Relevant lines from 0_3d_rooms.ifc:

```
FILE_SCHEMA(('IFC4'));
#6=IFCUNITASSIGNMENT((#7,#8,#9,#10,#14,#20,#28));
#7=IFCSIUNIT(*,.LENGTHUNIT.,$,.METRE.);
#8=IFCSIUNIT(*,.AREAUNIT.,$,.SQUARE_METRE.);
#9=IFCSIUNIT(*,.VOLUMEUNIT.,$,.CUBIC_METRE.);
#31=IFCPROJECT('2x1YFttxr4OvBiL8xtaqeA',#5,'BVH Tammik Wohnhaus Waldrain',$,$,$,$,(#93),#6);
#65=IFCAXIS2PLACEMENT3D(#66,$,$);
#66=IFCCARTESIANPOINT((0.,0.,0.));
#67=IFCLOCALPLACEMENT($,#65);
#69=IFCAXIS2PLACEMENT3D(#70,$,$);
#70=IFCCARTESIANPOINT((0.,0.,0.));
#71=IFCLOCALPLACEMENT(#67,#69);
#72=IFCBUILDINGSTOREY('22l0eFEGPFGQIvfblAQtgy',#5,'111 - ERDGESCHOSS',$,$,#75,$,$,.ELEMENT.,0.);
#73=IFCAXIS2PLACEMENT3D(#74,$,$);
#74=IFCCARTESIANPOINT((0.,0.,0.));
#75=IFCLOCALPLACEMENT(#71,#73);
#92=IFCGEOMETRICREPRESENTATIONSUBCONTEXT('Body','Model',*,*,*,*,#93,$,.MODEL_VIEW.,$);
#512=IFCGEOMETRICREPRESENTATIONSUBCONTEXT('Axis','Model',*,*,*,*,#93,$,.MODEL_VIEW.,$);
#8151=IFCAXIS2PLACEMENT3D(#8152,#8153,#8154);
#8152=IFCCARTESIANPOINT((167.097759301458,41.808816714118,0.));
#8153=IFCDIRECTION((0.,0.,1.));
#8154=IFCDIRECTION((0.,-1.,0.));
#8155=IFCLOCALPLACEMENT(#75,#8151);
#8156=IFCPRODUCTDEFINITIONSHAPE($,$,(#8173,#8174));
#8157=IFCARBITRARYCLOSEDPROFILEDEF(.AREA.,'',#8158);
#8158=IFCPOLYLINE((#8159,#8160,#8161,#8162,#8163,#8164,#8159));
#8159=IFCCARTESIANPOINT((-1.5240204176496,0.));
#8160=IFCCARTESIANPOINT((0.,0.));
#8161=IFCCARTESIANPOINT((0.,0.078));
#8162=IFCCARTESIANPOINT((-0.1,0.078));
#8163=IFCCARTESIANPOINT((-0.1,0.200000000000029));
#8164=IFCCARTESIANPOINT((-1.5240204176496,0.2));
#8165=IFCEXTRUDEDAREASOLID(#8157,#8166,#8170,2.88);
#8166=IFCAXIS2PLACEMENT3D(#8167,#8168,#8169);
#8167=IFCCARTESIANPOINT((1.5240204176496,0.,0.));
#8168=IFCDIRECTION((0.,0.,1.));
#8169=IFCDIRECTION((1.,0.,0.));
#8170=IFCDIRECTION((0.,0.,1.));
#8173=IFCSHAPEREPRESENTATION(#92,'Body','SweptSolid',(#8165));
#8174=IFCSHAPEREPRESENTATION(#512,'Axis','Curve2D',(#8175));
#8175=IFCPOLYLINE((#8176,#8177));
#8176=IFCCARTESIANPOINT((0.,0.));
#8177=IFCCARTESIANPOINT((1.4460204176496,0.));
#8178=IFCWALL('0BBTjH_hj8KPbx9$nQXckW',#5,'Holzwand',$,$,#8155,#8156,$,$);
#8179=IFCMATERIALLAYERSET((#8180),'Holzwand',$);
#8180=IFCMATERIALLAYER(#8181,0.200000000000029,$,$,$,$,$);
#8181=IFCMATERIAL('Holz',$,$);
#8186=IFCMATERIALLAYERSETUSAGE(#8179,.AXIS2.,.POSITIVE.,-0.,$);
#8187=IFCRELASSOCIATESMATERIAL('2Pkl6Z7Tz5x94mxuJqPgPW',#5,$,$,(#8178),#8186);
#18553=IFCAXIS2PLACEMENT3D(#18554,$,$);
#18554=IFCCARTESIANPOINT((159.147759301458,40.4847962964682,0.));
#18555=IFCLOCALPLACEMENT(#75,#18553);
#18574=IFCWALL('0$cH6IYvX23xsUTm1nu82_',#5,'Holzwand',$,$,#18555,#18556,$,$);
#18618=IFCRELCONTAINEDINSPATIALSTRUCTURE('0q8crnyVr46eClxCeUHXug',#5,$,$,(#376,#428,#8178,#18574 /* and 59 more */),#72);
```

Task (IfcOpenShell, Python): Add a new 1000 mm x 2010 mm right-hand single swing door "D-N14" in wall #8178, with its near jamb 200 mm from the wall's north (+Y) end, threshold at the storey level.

```python
import numpy as np
import ifcopenshell
import ifcopenshell.api.feature
import ifcopenshell.api.geometry
import ifcopenshell.api.root
import ifcopenshell.api.spatial
import ifcopenshell.geom
import ifcopenshell.util.element
import ifcopenshell.util.placement
import ifcopenshell.util.representation
import ifcopenshell.util.shape
import ifcopenshell.util.unit

model = ifcopenshell.open("0_3d_rooms.ifc")
unit_scale = ifcopenshell.util.unit.calculate_unit_scale(model)
settings = ifcopenshell.geom.settings()


def volume(element):
    """Net volume in cubic metres, openings subtracted."""
    shape = ifcopenshell.geom.create_shape(settings, element)
    return ifcopenshell.util.shape.get_volume(shape.geometry)


wall = model.by_guid("0BBTjH_hj8KPbx9$nQXckW")
storey = ifcopenshell.util.element.get_container(wall, ifc_class="IfcBuildingStorey")
context = ifcopenshell.util.representation.get_context(model, "Model", "Body", "MODEL_VIEW")
before = volume(wall)

width, height, from_end, sill = 1, 2.01, 0.2, 0.0  # metres

# The wall runs along its own X axis, and the end named is its -X end.
wall_shape = ifcopenshell.geom.create_shape(settings, wall)
x, y, z = ifcopenshell.util.shape.get_vertices(wall_shape.geometry).T
start = x.min() + from_end
face, thickness = float(y.min()), float(y.max() - y.min())
wall_matrix = ifcopenshell.util.placement.get_local_placement(wall.ObjectPlacement)
level = ifcopenshell.util.placement.get_local_placement(storey.ObjectPlacement)[2, 3]


def in_wall(x, y):
    """Placement at x, y metres in the wall's axes, at sill height."""
    matrix = wall_matrix.copy()
    matrix[:, 3] = wall_matrix @ np.array([x / unit_scale, y / unit_scale, 0.0, 1.0])
    matrix[2, 3] = level + sill / unit_scale
    return matrix


# Opening: a box that overshoots both wall faces by 50 mm.
opening = ifcopenshell.api.root.create_entity(model, ifc_class="IfcOpeningElement", predefined_type="OPENING")
box = ifcopenshell.api.geometry.add_wall_representation(
    model, context=context, length=width, height=height, thickness=thickness + 0.1
)
ifcopenshell.api.geometry.assign_representation(model, product=opening, representation=box)
ifcopenshell.api.geometry.edit_object_placement(model, product=opening, matrix=in_wall(start, face - 0.05), is_si=False)
ifcopenshell.api.feature.add_feature(model, feature=opening, element=wall)

door = ifcopenshell.api.root.create_entity(model, ifc_class="IfcDoor", name="D-N14", predefined_type="DOOR")
door.OverallWidth, door.OverallHeight = width / unit_scale, height / unit_scale
door.OperationType = "SINGLE_SWING_RIGHT"
body = ifcopenshell.api.geometry.add_door_representation(
    model,
    context=context,
    overall_width=door.OverallWidth,
    overall_height=door.OverallHeight,
    operation_type="SINGLE_SWING_RIGHT",
    lining_properties={"LiningDepth": thickness / unit_scale, "ThresholdDepth": thickness / unit_scale},
)
ifcopenshell.api.geometry.assign_representation(model, product=door, representation=body)
ifcopenshell.api.spatial.assign_container(model, products=[door], relating_structure=storey)
ifcopenshell.api.feature.add_filling(model, opening=opening, element=door)

# The lining spans the wall, so the door starts at the wall face.
ifcopenshell.api.geometry.edit_object_placement(model, product=door, matrix=in_wall(start, face), is_si=False)

after = volume(wall)

print(f"wall volume {before:.3f} -> {after:.3f} m3")

model.write("0_3d_rooms-out.ifc")
```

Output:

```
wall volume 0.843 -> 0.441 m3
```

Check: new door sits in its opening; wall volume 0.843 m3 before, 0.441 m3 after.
